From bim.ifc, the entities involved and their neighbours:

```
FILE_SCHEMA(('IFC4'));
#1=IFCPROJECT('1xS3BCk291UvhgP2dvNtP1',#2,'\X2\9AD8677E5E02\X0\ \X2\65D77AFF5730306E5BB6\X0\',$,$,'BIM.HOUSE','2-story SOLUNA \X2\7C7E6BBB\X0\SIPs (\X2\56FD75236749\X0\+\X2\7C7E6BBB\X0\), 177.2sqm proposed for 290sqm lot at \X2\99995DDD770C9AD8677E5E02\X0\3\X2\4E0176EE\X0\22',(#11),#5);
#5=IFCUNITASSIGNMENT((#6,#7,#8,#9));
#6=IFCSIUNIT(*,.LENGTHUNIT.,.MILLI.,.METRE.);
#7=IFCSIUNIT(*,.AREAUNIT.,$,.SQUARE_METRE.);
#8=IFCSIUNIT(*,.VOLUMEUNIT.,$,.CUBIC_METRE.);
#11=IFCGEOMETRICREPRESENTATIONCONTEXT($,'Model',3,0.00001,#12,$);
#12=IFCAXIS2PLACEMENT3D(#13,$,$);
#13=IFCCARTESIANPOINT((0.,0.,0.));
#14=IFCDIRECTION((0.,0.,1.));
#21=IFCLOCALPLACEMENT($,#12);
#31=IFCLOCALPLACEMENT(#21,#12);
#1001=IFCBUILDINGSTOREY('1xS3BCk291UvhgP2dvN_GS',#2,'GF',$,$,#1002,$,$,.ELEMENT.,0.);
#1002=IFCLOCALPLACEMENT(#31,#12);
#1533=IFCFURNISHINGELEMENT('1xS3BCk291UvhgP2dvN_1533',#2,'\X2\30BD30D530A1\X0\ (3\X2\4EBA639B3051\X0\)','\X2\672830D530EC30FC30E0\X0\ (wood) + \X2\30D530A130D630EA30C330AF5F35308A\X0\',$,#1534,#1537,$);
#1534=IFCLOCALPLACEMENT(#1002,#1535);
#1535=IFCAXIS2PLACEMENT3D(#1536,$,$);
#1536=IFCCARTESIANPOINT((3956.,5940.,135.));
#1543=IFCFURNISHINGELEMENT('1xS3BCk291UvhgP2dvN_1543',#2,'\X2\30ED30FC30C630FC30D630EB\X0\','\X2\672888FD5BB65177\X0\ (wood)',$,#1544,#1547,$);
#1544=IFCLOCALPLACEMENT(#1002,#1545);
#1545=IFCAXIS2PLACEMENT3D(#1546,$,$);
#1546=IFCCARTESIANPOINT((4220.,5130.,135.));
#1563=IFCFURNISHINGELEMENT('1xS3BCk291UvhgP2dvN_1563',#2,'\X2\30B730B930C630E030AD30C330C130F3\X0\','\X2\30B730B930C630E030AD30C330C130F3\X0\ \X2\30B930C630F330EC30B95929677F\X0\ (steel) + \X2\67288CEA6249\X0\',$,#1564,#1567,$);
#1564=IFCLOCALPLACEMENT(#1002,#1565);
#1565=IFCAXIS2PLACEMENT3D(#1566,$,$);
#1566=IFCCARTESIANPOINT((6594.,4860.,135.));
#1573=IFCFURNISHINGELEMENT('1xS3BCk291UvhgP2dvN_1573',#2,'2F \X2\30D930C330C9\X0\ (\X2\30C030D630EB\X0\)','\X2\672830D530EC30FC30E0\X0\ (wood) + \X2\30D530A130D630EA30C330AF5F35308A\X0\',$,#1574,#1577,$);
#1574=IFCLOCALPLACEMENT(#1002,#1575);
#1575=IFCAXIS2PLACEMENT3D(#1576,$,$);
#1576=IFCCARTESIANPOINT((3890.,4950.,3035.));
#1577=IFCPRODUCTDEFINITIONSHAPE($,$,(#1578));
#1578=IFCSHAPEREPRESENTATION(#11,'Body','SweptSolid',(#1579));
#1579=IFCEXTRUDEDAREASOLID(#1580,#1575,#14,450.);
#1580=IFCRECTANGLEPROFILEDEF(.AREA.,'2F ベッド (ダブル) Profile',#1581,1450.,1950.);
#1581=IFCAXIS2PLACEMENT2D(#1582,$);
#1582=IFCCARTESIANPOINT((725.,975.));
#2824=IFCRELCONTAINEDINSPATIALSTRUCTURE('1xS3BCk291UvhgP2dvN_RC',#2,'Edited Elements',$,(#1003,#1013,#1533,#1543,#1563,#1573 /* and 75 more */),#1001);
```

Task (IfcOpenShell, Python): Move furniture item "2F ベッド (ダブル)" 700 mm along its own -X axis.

```python
import ifcopenshell
import ifcopenshell.api.geometry
import ifcopenshell.util.placement
import ifcopenshell.util.unit

model = ifcopenshell.open("bim.ifc")
unit_scale = ifcopenshell.util.unit.calculate_unit_scale(model)

item = model.by_guid("1xS3BCk291UvhgP2dvN_1573")
matrix = ifcopenshell.util.placement.get_local_placement(item.ObjectPlacement)
matrix[:3, 3] -= matrix[:3, 0] * 0.7 / unit_scale
ifcopenshell.api.geometry.edit_object_placement(model, product=item, matrix=matrix, is_si=False)

print(ifcopenshell.util.placement.get_local_placement(item.ObjectPlacement).round(3) + 0.0)

model.write("bim_edited.ifc")
```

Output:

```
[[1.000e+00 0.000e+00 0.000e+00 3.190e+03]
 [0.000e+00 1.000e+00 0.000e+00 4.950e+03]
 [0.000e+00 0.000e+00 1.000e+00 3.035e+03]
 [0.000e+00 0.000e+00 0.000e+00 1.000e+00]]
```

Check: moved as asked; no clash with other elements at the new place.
